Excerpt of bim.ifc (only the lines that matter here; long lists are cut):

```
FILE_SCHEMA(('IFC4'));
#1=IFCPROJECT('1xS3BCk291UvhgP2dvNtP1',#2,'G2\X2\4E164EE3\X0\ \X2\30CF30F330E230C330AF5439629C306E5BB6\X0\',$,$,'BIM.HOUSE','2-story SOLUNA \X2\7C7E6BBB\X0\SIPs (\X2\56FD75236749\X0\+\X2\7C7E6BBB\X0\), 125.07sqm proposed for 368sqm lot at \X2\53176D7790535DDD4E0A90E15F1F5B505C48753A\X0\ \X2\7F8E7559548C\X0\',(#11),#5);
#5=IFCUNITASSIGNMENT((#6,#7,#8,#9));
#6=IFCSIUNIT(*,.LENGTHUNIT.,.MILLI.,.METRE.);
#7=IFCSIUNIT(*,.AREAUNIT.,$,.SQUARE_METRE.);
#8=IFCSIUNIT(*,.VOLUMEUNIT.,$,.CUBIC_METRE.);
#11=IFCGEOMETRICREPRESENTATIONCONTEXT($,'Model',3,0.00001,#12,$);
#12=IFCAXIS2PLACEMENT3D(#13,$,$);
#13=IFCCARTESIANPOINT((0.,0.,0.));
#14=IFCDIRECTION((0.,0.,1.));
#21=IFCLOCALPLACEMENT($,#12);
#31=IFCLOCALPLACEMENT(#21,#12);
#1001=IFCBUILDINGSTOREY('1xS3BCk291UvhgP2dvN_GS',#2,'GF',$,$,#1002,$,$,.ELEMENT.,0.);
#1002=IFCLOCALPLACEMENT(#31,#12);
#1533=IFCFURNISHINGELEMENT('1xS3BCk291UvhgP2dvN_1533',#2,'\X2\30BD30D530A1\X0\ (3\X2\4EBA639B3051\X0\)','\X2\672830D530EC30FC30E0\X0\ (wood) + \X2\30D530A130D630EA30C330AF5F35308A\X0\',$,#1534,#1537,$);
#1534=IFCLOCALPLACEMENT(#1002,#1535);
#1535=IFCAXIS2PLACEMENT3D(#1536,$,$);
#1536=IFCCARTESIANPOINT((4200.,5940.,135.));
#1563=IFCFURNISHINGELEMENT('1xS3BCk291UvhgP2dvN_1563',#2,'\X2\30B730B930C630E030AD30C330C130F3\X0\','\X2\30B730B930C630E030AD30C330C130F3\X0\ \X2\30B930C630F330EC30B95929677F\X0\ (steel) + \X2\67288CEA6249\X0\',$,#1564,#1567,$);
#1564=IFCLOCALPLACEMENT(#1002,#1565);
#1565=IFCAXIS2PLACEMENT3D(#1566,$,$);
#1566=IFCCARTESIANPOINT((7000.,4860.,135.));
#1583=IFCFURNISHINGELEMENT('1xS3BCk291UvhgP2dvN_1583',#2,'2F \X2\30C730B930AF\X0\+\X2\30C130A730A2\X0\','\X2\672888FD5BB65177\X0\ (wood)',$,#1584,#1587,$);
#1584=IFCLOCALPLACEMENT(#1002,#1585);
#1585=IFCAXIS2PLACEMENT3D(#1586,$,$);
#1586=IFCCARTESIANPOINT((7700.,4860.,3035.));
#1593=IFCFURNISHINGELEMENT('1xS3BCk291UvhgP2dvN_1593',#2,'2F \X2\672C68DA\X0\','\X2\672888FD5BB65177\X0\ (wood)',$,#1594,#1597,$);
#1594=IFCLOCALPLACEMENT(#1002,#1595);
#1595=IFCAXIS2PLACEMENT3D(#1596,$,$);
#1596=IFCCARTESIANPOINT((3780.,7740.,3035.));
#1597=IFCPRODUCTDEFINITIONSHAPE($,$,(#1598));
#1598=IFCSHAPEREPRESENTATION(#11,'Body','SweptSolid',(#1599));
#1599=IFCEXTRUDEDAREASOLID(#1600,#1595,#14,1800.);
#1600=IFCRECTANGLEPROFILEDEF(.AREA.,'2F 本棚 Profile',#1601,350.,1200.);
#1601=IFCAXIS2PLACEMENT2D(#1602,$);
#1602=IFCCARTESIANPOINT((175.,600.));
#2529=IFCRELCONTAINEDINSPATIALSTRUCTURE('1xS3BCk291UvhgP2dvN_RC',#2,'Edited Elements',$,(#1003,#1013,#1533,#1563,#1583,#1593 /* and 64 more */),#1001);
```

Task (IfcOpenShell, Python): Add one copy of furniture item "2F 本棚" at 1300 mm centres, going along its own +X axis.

```python
import ifcopenshell
import ifcopenshell.api.geometry
import ifcopenshell.api.root
import ifcopenshell.util.element
import ifcopenshell.util.placement

model = ifcopenshell.open("bim.ifc")


def reuse_history(source, copy):
    """copy_class also copies each property set's owner history, people and application; keep the originals."""
    for rel in copy.IsDefinedBy:
        if rel.is_a("IfcRelDefinesByProperties") and (history := rel.RelatingPropertyDefinition.OwnerHistory):
            rel.RelatingPropertyDefinition.OwnerHistory = source.OwnerHistory
            ifcopenshell.util.element.remove_deep2(model, history)


source = model.by_guid("1xS3BCk291UvhgP2dvN_1593")
base = ifcopenshell.util.placement.get_local_placement(source.ObjectPlacement)
step = base[:3, 0] * 1300.0

for i in range(1, 2):
    copy = ifcopenshell.api.root.copy_class(model, product=source)
    copy.Representation = ifcopenshell.util.element.copy_deep(
        model, source.Representation, exclude=["IfcGeometricRepresentationContext", "IfcRepresentationMap"]
    )
    reuse_history(source, copy)
    matrix = base.copy()
    matrix[:3, 3] += i * step
    print("added at", matrix[:3, 3].round(3) + 0.0)
    ifcopenshell.api.geometry.edit_object_placement(model, product=copy, matrix=matrix, is_si=False)

model.write("bim_v2.ifc")
```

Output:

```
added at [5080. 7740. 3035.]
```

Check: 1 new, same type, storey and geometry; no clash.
